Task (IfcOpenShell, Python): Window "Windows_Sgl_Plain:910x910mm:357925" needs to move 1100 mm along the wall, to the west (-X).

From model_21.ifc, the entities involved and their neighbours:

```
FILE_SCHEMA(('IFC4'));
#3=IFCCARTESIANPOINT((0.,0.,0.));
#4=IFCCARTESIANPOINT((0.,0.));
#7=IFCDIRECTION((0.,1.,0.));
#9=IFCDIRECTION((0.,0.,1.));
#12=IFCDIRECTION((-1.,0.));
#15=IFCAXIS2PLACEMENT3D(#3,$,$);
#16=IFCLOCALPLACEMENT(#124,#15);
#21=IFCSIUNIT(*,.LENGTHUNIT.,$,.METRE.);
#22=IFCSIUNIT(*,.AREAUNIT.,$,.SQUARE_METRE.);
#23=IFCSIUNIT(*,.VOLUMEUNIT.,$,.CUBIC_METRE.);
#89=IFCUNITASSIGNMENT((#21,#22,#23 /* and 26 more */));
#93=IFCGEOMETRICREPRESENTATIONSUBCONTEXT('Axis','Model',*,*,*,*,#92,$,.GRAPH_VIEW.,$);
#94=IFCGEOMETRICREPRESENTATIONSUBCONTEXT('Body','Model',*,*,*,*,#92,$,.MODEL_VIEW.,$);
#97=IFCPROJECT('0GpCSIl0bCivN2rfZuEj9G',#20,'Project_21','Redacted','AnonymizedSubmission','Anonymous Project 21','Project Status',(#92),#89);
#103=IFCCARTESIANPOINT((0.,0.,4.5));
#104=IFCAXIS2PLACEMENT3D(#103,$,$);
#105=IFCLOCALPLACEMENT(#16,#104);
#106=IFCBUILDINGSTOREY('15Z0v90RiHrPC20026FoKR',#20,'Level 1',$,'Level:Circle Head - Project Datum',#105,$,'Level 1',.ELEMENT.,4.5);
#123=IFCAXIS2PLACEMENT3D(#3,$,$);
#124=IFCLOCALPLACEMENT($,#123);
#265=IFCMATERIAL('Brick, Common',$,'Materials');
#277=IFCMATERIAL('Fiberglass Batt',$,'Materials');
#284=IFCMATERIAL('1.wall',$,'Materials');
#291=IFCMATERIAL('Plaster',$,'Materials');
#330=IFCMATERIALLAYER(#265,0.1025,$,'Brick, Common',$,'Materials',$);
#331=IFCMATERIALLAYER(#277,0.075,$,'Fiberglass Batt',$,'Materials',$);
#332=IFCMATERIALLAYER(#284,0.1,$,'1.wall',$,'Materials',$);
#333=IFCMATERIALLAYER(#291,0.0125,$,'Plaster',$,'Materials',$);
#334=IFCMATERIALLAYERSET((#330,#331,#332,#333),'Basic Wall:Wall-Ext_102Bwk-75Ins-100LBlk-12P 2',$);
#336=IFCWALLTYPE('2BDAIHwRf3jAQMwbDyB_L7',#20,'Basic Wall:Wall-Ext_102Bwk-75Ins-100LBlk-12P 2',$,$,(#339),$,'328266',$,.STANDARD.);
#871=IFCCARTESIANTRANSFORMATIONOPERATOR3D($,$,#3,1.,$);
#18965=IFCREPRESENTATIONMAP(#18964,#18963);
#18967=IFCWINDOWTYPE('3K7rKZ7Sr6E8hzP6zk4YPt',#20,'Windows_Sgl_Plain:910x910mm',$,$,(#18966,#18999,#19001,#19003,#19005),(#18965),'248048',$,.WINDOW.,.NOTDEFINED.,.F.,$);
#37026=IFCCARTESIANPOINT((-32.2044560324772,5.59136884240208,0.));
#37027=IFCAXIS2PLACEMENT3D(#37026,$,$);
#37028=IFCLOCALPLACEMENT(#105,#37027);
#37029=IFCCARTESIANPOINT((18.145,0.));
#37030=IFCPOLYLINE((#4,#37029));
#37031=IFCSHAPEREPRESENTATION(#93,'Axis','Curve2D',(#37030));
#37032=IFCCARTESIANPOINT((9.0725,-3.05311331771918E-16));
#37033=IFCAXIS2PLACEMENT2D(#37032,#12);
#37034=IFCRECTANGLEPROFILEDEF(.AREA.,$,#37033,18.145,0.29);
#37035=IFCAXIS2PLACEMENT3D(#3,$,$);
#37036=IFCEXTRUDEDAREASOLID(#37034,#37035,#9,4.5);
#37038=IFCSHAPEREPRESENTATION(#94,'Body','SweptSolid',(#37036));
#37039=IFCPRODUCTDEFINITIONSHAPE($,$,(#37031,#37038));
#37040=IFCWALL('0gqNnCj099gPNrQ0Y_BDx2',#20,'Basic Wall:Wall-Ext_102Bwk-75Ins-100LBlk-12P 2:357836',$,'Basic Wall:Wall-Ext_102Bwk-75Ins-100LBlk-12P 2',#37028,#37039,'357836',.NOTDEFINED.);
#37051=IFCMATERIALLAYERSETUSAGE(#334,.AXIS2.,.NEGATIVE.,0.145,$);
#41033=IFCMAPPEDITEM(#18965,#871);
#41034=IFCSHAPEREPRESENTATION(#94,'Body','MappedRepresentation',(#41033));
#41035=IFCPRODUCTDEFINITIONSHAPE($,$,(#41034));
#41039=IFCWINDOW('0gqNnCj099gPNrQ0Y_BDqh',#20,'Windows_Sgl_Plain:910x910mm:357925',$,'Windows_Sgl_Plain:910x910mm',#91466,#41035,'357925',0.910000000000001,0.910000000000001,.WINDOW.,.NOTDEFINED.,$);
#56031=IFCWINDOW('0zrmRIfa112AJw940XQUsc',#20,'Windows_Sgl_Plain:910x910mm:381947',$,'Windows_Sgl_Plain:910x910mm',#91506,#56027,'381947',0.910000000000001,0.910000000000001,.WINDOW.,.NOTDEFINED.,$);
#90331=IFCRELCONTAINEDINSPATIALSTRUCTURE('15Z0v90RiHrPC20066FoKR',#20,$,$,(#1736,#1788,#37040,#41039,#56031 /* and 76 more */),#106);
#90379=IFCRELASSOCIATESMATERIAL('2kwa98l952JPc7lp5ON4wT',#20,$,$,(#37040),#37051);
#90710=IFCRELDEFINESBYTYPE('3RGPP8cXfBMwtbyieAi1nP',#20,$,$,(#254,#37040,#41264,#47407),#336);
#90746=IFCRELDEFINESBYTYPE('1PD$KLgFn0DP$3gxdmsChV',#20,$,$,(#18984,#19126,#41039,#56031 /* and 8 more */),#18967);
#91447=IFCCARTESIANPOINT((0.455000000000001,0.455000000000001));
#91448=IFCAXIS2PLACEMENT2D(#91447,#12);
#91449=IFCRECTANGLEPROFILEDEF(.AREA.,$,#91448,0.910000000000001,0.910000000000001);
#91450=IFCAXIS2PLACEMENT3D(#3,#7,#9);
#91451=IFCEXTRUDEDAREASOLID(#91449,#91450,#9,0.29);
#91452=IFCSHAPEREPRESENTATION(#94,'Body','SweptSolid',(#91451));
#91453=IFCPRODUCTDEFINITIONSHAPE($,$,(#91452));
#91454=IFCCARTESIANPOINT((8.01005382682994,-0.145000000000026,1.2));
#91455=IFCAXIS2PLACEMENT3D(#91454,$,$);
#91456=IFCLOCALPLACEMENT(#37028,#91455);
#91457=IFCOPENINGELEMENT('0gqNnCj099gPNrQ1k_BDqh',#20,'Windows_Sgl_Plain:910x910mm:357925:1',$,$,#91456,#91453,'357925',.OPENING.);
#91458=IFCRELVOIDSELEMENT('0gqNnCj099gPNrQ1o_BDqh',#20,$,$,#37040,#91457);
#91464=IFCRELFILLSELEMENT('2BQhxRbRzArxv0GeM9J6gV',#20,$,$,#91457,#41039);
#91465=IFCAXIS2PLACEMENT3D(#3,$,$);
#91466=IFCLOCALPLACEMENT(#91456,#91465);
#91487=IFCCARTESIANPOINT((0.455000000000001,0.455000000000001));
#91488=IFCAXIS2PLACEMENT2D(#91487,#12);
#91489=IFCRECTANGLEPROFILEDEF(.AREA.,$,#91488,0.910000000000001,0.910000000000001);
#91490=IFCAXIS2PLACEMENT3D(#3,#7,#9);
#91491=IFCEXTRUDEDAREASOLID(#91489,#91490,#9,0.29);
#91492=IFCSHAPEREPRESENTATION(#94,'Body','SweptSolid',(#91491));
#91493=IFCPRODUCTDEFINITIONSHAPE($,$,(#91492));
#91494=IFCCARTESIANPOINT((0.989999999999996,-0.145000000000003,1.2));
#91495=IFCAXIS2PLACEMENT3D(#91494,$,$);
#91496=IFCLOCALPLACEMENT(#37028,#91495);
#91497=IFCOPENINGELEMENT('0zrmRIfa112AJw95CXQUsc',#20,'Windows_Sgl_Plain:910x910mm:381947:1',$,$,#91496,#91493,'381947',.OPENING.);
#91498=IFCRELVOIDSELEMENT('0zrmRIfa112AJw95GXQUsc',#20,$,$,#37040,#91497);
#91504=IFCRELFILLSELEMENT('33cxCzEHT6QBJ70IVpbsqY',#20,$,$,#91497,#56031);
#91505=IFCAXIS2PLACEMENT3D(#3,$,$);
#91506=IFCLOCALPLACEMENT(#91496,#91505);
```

```python
import ifcopenshell
import ifcopenshell.api.geometry
import ifcopenshell.util.placement

model = ifcopenshell.open("model_21.ifc")

window = model.by_guid("0gqNnCj099gPNrQ0Y_BDqh")
opening = window.FillsVoids[0].RelatingOpeningElement
wall = opening.VoidsElements[0].RelatingBuildingElement

wall_matrix = ifcopenshell.util.placement.get_local_placement(wall.ObjectPlacement)
shift = wall_matrix[:3, 0] * -1.1
before = ifcopenshell.util.placement.get_local_placement(window.ObjectPlacement)[:3, 3].copy()

# The window is placed relative to its opening, so it follows when the opening moves.
matrix = ifcopenshell.util.placement.get_local_placement(opening.ObjectPlacement)
matrix[:3, 3] += shift
ifcopenshell.api.geometry.edit_object_placement(
    model, product=opening, matrix=matrix, is_si=False, should_transform_children=True
)

after = ifcopenshell.util.placement.get_local_placement(window.ObjectPlacement)[:3, 3]
print("window moved by", (after - before).round(3) + 0.0)

model.write("model_21-out.ifc")
```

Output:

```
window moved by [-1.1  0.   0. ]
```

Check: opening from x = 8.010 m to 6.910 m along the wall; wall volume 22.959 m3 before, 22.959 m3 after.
